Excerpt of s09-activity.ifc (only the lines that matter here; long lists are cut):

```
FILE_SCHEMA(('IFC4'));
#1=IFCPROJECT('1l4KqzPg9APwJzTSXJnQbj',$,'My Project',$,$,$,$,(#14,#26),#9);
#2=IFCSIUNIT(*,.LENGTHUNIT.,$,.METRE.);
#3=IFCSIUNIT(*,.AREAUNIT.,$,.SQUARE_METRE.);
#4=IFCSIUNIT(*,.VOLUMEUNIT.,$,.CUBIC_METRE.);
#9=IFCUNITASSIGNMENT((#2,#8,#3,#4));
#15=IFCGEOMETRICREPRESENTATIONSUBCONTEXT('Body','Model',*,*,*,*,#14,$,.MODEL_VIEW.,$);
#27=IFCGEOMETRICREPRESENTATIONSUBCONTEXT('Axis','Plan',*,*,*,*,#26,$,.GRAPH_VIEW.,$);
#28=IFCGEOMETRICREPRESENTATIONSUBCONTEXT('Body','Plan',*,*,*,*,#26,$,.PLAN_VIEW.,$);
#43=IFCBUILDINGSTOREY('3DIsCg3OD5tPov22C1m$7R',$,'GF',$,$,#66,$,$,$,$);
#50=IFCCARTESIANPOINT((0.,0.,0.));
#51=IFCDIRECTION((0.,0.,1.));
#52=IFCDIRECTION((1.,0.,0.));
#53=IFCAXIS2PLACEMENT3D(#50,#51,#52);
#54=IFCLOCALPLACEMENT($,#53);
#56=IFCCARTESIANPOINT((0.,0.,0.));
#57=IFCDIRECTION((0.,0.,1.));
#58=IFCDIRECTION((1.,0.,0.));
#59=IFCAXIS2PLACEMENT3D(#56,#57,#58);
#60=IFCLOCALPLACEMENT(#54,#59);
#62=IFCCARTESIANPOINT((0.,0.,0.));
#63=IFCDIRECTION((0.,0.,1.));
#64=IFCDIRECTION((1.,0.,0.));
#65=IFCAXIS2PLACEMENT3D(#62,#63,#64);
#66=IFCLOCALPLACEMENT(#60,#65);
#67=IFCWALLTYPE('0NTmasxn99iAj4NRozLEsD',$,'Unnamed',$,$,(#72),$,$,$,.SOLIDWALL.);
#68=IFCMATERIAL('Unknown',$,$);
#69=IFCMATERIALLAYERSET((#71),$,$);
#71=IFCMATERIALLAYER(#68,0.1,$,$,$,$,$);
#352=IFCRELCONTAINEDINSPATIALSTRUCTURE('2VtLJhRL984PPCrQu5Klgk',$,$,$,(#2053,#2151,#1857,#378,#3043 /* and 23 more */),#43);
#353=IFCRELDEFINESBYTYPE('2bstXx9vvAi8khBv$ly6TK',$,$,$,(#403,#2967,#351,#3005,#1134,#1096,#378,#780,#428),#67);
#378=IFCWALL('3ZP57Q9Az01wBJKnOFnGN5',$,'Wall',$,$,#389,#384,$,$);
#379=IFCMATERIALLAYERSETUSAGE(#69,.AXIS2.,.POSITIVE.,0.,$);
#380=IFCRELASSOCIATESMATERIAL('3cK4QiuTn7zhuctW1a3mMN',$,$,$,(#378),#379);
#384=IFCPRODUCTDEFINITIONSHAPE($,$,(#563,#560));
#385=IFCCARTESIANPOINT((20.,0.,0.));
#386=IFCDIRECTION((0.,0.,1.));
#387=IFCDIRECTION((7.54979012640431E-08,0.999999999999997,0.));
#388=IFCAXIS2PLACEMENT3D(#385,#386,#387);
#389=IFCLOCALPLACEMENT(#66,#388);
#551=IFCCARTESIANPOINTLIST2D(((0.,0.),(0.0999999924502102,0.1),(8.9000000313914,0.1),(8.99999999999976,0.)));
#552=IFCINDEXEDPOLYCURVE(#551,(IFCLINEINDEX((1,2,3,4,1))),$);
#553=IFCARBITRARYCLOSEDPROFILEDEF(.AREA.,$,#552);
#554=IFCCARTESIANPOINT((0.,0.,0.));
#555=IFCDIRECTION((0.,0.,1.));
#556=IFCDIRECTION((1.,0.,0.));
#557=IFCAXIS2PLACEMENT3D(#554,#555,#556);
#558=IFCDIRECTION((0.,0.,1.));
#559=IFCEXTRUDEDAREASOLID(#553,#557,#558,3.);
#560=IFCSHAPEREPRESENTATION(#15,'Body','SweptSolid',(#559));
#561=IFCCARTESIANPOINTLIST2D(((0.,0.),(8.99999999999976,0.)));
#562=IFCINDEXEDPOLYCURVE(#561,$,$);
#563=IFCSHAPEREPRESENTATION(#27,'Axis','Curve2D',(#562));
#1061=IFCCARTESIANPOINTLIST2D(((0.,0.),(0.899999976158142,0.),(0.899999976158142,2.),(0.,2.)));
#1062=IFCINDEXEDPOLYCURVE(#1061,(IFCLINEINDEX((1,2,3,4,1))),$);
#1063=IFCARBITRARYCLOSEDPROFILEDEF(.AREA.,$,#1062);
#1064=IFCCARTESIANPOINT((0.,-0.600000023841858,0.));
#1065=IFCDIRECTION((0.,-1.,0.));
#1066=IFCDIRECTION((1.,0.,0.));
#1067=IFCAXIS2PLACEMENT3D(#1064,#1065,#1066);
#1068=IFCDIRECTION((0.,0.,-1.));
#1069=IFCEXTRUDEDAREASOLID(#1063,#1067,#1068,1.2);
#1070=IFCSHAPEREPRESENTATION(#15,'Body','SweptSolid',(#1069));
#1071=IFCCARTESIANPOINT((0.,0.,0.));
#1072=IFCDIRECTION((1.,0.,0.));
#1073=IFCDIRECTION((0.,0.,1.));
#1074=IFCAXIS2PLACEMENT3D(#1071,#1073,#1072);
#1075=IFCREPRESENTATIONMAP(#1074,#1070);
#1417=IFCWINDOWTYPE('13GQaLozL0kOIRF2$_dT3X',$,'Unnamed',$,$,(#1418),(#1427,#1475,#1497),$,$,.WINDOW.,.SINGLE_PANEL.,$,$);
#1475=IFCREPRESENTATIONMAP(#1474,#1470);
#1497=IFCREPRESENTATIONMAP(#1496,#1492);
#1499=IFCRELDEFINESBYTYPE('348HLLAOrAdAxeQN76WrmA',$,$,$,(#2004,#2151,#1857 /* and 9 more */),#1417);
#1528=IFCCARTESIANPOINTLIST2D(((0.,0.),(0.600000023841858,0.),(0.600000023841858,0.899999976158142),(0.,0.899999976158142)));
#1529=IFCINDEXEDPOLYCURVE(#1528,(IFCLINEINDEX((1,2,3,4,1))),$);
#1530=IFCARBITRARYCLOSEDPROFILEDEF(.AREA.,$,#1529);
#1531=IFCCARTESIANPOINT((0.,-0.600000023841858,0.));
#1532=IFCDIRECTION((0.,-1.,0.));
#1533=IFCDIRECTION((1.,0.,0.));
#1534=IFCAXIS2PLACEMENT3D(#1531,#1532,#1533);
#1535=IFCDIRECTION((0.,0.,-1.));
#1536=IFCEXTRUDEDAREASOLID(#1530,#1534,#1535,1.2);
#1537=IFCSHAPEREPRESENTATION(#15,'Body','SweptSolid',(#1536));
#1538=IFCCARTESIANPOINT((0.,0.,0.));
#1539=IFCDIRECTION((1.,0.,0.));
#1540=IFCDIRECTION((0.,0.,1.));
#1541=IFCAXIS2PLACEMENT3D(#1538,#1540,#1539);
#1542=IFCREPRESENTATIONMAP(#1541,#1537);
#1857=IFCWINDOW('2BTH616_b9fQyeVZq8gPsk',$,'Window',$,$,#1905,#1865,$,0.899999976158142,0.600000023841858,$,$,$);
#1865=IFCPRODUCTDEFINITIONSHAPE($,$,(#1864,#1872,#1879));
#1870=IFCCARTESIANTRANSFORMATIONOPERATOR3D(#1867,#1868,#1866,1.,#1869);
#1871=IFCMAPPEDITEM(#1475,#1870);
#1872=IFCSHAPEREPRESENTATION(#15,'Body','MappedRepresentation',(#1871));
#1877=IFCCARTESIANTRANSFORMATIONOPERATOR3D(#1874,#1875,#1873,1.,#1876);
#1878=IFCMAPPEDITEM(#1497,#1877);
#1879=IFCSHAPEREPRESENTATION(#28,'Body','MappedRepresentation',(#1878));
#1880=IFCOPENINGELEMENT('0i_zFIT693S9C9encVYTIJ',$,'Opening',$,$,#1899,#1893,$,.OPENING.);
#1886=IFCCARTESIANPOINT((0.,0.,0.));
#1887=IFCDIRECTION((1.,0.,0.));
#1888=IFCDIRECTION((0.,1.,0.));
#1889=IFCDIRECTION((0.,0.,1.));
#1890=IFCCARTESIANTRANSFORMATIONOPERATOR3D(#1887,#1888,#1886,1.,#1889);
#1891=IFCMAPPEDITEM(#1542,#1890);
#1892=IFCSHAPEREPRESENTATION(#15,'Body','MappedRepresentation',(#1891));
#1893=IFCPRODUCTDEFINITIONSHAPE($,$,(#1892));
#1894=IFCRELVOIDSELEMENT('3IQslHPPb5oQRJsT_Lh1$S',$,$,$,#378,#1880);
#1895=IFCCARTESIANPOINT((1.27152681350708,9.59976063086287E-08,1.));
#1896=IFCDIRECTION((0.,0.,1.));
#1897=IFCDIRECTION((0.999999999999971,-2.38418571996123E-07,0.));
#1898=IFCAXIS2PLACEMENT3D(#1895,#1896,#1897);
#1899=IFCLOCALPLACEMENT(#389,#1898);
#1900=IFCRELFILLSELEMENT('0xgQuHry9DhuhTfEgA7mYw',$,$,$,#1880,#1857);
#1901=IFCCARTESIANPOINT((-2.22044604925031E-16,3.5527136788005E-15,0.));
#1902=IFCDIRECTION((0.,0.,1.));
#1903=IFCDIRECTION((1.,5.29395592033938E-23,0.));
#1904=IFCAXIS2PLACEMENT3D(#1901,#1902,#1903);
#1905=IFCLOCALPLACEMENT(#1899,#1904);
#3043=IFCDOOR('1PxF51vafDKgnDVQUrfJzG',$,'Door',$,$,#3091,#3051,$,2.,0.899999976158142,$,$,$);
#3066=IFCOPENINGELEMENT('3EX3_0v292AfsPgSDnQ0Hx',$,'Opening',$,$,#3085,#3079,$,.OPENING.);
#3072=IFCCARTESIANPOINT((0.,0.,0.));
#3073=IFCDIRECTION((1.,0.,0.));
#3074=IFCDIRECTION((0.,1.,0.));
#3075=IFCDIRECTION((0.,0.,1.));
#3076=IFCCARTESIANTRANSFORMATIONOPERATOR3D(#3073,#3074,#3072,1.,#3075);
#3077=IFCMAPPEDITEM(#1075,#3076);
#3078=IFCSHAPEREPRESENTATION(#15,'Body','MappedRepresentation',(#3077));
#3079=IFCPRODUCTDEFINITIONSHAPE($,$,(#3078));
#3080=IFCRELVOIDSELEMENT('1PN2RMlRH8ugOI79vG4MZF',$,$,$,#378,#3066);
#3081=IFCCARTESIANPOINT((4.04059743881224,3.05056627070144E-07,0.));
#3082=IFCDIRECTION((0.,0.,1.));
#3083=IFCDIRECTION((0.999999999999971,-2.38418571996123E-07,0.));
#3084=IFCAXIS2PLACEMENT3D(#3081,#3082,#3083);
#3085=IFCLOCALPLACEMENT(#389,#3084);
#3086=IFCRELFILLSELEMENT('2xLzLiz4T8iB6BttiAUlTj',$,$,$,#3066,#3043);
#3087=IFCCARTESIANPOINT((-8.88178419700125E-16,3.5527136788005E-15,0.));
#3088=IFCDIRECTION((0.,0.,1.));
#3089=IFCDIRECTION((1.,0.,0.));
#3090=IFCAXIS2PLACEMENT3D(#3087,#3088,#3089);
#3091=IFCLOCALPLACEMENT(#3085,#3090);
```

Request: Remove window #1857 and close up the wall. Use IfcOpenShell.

```python
import ifcopenshell
import ifcopenshell.api.feature
import ifcopenshell.api.root
import ifcopenshell.geom
import ifcopenshell.util.shape

model = ifcopenshell.open("s09-activity.ifc")
settings = ifcopenshell.geom.settings()


def volume(element):
    """Net volume in cubic metres, openings subtracted."""
    shape = ifcopenshell.geom.create_shape(settings, element)
    return ifcopenshell.util.shape.get_volume(shape.geometry)


window = model.by_guid("2BTH616_b9fQyeVZq8gPsk")
opening = window.FillsVoids[0].RelatingOpeningElement
wall = opening.VoidsElements[0].RelatingBuildingElement
before = volume(wall)

ifcopenshell.api.root.remove_product(model, product=window)
ifcopenshell.api.feature.remove_feature(model, feature=opening)

after = volume(wall)

print(f"wall volume {before:.3f} -> {after:.3f} m3")

model.write("s09-activity-out.ifc")
```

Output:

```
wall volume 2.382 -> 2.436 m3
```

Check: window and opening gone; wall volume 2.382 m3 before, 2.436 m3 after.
